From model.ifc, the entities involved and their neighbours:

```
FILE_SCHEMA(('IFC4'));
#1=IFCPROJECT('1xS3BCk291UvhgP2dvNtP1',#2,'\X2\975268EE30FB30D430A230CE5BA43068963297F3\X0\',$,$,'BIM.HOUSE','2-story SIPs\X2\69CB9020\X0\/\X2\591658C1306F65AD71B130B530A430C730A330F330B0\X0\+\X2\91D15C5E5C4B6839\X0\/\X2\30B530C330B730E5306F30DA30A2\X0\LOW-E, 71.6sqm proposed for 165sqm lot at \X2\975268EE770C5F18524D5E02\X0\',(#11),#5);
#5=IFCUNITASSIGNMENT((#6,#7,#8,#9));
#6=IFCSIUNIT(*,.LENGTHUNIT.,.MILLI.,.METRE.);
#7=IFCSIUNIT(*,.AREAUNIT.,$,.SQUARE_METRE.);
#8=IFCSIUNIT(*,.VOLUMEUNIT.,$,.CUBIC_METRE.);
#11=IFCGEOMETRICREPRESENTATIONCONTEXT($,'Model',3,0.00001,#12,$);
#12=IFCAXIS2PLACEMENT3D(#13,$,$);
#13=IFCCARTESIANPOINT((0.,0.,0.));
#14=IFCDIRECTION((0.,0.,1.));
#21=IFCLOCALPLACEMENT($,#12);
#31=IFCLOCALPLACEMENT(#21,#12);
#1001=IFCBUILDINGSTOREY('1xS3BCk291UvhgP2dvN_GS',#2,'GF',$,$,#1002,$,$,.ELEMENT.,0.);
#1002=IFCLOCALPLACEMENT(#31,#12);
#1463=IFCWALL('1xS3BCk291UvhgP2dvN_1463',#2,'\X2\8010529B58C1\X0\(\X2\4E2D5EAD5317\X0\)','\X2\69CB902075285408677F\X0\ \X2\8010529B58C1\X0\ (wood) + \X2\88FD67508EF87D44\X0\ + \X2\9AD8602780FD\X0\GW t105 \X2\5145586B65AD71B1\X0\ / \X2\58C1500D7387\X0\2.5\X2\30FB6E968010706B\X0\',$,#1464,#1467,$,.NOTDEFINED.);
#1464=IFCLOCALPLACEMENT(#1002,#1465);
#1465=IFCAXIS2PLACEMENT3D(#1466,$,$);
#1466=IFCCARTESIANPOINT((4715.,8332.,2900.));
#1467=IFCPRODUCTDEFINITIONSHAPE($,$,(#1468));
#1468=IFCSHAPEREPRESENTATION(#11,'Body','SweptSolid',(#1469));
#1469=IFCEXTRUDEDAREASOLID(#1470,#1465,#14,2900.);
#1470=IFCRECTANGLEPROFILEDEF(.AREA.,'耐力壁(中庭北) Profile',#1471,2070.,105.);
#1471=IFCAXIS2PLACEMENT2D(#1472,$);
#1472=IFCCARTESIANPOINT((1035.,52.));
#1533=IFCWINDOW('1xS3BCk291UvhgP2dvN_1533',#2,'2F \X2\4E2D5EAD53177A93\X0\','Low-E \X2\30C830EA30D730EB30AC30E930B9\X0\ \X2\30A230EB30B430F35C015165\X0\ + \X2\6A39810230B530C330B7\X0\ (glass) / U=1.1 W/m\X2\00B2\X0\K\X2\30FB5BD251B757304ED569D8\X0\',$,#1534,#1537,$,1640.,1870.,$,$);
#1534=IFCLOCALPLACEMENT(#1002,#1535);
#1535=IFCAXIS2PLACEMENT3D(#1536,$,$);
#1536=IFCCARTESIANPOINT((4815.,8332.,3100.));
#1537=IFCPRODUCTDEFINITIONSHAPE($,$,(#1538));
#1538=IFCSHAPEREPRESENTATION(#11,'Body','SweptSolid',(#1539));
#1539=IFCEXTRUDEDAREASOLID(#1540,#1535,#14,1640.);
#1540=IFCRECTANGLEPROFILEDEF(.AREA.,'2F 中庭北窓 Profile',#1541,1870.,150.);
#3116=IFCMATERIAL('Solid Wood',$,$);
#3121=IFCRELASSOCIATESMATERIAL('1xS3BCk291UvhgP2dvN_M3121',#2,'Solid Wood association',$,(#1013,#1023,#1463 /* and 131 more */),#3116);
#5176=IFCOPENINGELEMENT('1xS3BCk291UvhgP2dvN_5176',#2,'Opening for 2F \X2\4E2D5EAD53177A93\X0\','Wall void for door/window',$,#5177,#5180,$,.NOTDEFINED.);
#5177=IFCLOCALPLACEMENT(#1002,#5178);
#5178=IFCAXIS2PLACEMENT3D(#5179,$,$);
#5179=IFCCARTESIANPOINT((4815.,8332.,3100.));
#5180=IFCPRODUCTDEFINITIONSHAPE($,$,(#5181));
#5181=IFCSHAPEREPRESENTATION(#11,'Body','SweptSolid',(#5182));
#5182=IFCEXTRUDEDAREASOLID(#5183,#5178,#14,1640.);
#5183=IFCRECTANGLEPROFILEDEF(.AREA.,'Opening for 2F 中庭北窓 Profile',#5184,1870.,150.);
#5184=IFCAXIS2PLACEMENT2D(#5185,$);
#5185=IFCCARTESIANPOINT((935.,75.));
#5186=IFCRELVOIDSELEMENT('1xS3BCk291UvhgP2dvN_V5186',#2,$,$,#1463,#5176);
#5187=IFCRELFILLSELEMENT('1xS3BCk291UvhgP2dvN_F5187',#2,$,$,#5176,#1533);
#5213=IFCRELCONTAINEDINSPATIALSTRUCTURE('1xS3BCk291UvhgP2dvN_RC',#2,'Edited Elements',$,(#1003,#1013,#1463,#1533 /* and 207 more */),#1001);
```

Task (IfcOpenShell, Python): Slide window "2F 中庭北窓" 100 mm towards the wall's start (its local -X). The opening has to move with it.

```python
import ifcopenshell
import ifcopenshell.api.geometry
import ifcopenshell.util.placement
import ifcopenshell.util.unit

model = ifcopenshell.open("model.ifc")
unit_scale = ifcopenshell.util.unit.calculate_unit_scale(model)

window = model.by_guid("1xS3BCk291UvhgP2dvN_1533")
opening = window.FillsVoids[0].RelatingOpeningElement
wall = opening.VoidsElements[0].RelatingBuildingElement

wall_matrix = ifcopenshell.util.placement.get_local_placement(wall.ObjectPlacement)
shift = wall_matrix[:3, 0] * -0.1 / unit_scale
before = ifcopenshell.util.placement.get_local_placement(window.ObjectPlacement)[:3, 3].copy()

# The window is not placed relative to its opening, so move both.
for product in (opening, window):
    matrix = ifcopenshell.util.placement.get_local_placement(product.ObjectPlacement)
    matrix[:3, 3] += shift
    ifcopenshell.api.geometry.edit_object_placement(model, product=product, matrix=matrix, is_si=False)

after = ifcopenshell.util.placement.get_local_placement(window.ObjectPlacement)[:3, 3]
print("window moved by", (after - before).round(3) + 0.0)

model.write("model_updated.ifc")
```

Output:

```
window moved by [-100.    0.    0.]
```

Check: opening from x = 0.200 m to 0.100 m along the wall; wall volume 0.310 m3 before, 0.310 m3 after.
